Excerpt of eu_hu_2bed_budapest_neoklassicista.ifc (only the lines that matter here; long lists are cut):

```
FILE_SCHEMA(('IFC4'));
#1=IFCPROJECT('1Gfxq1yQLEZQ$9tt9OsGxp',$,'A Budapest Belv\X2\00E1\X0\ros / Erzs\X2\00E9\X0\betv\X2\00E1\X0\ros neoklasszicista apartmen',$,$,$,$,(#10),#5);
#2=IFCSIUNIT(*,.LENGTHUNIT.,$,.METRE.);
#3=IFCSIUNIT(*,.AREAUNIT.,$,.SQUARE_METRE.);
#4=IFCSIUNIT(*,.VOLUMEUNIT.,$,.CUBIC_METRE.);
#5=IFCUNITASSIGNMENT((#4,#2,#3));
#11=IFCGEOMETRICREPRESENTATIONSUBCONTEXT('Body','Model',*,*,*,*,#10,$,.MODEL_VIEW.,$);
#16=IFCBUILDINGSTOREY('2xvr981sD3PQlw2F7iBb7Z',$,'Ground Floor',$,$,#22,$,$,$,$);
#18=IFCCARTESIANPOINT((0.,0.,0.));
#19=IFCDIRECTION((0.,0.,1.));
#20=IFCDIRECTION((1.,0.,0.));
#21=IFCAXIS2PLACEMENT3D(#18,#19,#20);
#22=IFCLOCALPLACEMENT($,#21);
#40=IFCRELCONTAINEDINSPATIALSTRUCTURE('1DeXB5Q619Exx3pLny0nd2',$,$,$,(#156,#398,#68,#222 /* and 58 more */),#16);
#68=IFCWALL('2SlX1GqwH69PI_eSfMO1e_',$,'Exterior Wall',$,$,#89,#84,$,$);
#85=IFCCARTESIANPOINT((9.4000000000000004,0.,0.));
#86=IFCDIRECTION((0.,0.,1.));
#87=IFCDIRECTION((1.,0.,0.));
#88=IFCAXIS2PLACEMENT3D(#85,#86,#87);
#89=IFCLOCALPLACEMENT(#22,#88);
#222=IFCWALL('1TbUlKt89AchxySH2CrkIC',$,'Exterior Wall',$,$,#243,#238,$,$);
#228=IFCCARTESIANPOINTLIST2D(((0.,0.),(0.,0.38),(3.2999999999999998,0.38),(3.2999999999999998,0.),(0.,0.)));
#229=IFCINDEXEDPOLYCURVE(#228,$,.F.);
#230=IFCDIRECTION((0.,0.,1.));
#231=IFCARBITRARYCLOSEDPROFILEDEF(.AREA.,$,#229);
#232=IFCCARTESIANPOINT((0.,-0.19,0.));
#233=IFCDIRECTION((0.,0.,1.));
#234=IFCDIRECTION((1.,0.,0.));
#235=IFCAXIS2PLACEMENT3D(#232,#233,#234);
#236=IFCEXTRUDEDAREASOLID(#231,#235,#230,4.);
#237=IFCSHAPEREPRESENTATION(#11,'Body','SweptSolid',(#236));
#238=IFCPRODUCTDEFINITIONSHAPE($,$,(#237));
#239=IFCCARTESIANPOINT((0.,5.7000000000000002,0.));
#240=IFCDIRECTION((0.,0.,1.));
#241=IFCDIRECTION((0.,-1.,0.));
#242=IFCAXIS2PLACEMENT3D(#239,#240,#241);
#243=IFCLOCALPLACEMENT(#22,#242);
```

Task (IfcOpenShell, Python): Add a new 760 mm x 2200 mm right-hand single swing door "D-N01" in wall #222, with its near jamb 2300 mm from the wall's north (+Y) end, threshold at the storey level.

```python
import numpy as np
import ifcopenshell
import ifcopenshell.api.feature
import ifcopenshell.api.geometry
import ifcopenshell.api.root
import ifcopenshell.api.spatial
import ifcopenshell.geom
import ifcopenshell.util.element
import ifcopenshell.util.placement
import ifcopenshell.util.representation
import ifcopenshell.util.shape
import ifcopenshell.util.unit

model = ifcopenshell.open("eu_hu_2bed_budapest_neoklassicista.ifc")
unit_scale = ifcopenshell.util.unit.calculate_unit_scale(model)
settings = ifcopenshell.geom.settings()


def volume(element):
    """Net volume in cubic metres, openings subtracted."""
    shape = ifcopenshell.geom.create_shape(settings, element)
    return ifcopenshell.util.shape.get_volume(shape.geometry)


wall = model.by_guid("1TbUlKt89AchxySH2CrkIC")
storey = ifcopenshell.util.element.get_container(wall, ifc_class="IfcBuildingStorey")
context = ifcopenshell.util.representation.get_context(model, "Model", "Body", "MODEL_VIEW")
before = volume(wall)

width, height, from_end, sill = 0.76, 2.2, 2.3, 0.0  # metres

# The wall runs along its own X axis, and the end named is its -X end.
wall_shape = ifcopenshell.geom.create_shape(settings, wall)
x, y, z = ifcopenshell.util.shape.get_vertices(wall_shape.geometry).T
start = x.min() + from_end
face, thickness = float(y.min()), float(y.max() - y.min())
wall_matrix = ifcopenshell.util.placement.get_local_placement(wall.ObjectPlacement)
level = ifcopenshell.util.placement.get_local_placement(storey.ObjectPlacement)[2, 3]


def in_wall(x, y):
    """Placement at x, y metres in the wall's axes, at sill height."""
    matrix = wall_matrix.copy()
    matrix[:, 3] = wall_matrix @ np.array([x / unit_scale, y / unit_scale, 0.0, 1.0])
    matrix[2, 3] = level + sill / unit_scale
    return matrix


# Opening: a box that overshoots both wall faces by 50 mm.
opening = ifcopenshell.api.root.create_entity(model, ifc_class="IfcOpeningElement", predefined_type="OPENING")
box = ifcopenshell.api.geometry.add_wall_representation(
    model, context=context, length=width, height=height, thickness=thickness + 0.1
)
ifcopenshell.api.geometry.assign_representation(model, product=opening, representation=box)
ifcopenshell.api.geometry.edit_object_placement(model, product=opening, matrix=in_wall(start, face - 0.05), is_si=False)
ifcopenshell.api.feature.add_feature(model, feature=opening, element=wall)

door = ifcopenshell.api.root.create_entity(model, ifc_class="IfcDoor", name="D-N01", predefined_type="DOOR")
door.OverallWidth, door.OverallHeight = width / unit_scale, height / unit_scale
door.OperationType = "SINGLE_SWING_RIGHT"
body = ifcopenshell.api.geometry.add_door_representation(
    model,
    context=context,
    overall_width=door.OverallWidth,
    overall_height=door.OverallHeight,
    operation_type="SINGLE_SWING_RIGHT",
    lining_properties={"LiningDepth": thickness / unit_scale, "ThresholdDepth": thickness / unit_scale},
)
ifcopenshell.api.geometry.assign_representation(model, product=door, representation=body)
ifcopenshell.api.spatial.assign_container(model, products=[door], relating_structure=storey)
ifcopenshell.api.feature.add_filling(model, opening=opening, element=door)

# The lining spans the wall, so the door starts at the wall face.
ifcopenshell.api.geometry.edit_object_placement(model, product=door, matrix=in_wall(start, face), is_si=False)

after = volume(wall)

print(f"wall volume {before:.3f} -> {after:.3f} m3")

model.write("eu_hu_2bed_budapest_neoklassicista_updated.ifc")
```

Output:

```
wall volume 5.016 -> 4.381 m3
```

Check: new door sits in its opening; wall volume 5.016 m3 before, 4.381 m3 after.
